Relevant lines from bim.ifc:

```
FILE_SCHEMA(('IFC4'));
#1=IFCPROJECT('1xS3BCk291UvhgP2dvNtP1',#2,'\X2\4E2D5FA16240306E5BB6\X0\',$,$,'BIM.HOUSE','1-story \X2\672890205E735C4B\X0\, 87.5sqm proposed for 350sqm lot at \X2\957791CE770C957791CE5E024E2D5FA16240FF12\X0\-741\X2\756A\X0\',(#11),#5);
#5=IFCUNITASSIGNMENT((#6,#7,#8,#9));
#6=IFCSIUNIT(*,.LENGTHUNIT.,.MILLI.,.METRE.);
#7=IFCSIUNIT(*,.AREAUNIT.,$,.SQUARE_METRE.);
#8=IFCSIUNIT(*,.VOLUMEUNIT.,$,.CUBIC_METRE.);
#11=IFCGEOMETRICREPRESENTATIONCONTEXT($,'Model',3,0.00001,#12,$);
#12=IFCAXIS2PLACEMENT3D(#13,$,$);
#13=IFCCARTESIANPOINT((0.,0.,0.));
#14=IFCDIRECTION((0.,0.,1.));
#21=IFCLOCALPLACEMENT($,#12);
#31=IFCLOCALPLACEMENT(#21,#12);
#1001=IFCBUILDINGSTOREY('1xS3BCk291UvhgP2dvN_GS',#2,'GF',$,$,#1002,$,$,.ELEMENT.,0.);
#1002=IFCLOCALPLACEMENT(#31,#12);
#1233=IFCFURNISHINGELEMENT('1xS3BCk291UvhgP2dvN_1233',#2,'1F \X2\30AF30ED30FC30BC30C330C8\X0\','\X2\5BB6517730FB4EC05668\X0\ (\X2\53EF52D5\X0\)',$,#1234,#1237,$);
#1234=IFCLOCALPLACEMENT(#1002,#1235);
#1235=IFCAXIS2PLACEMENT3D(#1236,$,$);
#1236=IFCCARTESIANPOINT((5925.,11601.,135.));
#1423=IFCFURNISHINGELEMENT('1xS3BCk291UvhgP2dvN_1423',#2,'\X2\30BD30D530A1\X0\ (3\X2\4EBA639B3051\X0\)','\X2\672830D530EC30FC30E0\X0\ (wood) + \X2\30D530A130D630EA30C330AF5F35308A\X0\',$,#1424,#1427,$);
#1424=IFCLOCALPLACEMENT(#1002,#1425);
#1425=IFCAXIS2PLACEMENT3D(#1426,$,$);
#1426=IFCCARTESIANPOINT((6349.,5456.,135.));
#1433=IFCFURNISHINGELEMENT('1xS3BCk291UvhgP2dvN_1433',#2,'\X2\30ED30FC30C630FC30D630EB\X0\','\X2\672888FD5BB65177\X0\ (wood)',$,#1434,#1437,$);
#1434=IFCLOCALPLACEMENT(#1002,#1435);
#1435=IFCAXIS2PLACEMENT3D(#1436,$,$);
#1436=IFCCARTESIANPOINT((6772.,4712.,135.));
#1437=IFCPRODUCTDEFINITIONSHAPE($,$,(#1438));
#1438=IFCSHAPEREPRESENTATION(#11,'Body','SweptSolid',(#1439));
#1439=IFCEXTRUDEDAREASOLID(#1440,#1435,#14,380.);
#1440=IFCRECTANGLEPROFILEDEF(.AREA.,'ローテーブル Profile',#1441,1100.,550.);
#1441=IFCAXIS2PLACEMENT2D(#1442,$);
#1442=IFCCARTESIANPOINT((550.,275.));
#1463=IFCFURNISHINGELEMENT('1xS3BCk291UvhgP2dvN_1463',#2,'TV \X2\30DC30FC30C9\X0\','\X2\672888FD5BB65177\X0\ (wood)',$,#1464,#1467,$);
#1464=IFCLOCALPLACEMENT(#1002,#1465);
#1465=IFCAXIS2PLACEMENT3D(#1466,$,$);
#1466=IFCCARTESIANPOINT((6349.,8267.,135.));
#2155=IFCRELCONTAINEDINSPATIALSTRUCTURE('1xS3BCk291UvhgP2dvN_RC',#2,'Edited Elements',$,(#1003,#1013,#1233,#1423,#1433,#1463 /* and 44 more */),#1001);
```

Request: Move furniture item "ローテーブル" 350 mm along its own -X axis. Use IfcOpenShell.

```python
import ifcopenshell
import ifcopenshell.api.geometry
import ifcopenshell.util.placement
import ifcopenshell.util.unit

model = ifcopenshell.open("bim.ifc")
unit_scale = ifcopenshell.util.unit.calculate_unit_scale(model)

item = model.by_guid("1xS3BCk291UvhgP2dvN_1433")
matrix = ifcopenshell.util.placement.get_local_placement(item.ObjectPlacement)
matrix[:3, 3] -= matrix[:3, 0] * 0.35 / unit_scale
ifcopenshell.api.geometry.edit_object_placement(model, product=item, matrix=matrix, is_si=False)

print(ifcopenshell.util.placement.get_local_placement(item.ObjectPlacement).round(3) + 0.0)

model.write("bim_edited.ifc")
```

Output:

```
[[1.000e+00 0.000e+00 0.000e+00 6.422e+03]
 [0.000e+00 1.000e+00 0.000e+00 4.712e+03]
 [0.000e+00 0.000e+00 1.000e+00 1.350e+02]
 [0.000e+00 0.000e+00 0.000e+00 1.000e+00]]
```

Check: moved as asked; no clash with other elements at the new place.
